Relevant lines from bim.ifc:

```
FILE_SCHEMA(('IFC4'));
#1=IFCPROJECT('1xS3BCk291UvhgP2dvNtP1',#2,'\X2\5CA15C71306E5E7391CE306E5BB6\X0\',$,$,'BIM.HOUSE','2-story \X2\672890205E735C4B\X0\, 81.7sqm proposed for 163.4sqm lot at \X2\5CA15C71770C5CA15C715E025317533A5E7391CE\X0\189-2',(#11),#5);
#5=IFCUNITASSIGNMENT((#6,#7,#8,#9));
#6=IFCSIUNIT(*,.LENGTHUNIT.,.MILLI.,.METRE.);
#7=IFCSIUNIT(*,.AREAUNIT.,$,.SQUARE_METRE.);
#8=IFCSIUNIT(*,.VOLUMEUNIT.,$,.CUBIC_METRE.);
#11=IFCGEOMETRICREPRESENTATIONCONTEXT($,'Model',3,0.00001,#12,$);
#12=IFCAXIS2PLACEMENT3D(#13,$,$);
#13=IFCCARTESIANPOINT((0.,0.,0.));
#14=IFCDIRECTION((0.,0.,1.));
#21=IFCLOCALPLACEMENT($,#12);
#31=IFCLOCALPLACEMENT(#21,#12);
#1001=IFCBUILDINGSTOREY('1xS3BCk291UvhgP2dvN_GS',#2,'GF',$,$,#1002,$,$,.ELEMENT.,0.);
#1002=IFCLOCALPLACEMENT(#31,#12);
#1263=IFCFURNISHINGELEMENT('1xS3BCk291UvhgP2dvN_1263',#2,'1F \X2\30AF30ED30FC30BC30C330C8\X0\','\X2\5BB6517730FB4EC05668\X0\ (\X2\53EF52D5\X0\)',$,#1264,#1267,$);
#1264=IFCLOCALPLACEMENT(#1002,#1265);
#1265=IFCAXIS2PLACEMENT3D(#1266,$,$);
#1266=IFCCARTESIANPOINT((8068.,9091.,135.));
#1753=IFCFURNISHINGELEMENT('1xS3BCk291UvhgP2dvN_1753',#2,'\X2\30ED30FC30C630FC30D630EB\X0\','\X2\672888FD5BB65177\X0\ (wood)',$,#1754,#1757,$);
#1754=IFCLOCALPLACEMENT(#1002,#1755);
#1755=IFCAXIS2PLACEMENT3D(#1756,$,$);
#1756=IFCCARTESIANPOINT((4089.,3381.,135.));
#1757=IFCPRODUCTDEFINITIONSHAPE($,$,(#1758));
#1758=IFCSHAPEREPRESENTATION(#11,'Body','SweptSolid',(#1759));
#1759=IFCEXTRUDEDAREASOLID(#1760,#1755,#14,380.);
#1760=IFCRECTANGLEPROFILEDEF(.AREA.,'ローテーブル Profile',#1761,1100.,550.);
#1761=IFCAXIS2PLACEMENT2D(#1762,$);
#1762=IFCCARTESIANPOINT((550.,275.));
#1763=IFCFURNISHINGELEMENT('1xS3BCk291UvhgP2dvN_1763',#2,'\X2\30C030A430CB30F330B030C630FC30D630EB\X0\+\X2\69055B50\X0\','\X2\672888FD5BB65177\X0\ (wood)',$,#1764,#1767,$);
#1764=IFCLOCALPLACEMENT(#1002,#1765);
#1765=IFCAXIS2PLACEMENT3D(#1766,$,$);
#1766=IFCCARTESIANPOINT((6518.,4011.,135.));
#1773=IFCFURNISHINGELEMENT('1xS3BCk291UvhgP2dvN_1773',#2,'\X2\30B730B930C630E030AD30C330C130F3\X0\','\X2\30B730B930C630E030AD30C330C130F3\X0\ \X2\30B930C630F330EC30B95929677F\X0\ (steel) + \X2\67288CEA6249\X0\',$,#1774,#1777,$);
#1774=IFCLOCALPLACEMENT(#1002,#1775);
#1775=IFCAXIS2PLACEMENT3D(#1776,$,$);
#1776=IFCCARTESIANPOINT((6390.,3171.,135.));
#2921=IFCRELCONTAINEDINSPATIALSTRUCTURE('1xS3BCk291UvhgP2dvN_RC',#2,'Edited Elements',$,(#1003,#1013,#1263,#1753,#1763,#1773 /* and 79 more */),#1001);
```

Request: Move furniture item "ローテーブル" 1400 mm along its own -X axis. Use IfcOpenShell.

```python
import ifcopenshell
import ifcopenshell.api.geometry
import ifcopenshell.util.placement
import ifcopenshell.util.unit

model = ifcopenshell.open("bim.ifc")
unit_scale = ifcopenshell.util.unit.calculate_unit_scale(model)

item = model.by_guid("1xS3BCk291UvhgP2dvN_1753")
matrix = ifcopenshell.util.placement.get_local_placement(item.ObjectPlacement)
matrix[:3, 3] -= matrix[:3, 0] * 1.4 / unit_scale
ifcopenshell.api.geometry.edit_object_placement(model, product=item, matrix=matrix, is_si=False)

print(ifcopenshell.util.placement.get_local_placement(item.ObjectPlacement).round(3) + 0.0)

model.write("bim_edited.ifc")
```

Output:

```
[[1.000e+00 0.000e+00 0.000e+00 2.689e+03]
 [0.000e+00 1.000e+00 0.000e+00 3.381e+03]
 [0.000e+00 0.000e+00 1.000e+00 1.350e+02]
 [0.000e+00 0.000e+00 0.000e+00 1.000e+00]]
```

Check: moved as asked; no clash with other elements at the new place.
